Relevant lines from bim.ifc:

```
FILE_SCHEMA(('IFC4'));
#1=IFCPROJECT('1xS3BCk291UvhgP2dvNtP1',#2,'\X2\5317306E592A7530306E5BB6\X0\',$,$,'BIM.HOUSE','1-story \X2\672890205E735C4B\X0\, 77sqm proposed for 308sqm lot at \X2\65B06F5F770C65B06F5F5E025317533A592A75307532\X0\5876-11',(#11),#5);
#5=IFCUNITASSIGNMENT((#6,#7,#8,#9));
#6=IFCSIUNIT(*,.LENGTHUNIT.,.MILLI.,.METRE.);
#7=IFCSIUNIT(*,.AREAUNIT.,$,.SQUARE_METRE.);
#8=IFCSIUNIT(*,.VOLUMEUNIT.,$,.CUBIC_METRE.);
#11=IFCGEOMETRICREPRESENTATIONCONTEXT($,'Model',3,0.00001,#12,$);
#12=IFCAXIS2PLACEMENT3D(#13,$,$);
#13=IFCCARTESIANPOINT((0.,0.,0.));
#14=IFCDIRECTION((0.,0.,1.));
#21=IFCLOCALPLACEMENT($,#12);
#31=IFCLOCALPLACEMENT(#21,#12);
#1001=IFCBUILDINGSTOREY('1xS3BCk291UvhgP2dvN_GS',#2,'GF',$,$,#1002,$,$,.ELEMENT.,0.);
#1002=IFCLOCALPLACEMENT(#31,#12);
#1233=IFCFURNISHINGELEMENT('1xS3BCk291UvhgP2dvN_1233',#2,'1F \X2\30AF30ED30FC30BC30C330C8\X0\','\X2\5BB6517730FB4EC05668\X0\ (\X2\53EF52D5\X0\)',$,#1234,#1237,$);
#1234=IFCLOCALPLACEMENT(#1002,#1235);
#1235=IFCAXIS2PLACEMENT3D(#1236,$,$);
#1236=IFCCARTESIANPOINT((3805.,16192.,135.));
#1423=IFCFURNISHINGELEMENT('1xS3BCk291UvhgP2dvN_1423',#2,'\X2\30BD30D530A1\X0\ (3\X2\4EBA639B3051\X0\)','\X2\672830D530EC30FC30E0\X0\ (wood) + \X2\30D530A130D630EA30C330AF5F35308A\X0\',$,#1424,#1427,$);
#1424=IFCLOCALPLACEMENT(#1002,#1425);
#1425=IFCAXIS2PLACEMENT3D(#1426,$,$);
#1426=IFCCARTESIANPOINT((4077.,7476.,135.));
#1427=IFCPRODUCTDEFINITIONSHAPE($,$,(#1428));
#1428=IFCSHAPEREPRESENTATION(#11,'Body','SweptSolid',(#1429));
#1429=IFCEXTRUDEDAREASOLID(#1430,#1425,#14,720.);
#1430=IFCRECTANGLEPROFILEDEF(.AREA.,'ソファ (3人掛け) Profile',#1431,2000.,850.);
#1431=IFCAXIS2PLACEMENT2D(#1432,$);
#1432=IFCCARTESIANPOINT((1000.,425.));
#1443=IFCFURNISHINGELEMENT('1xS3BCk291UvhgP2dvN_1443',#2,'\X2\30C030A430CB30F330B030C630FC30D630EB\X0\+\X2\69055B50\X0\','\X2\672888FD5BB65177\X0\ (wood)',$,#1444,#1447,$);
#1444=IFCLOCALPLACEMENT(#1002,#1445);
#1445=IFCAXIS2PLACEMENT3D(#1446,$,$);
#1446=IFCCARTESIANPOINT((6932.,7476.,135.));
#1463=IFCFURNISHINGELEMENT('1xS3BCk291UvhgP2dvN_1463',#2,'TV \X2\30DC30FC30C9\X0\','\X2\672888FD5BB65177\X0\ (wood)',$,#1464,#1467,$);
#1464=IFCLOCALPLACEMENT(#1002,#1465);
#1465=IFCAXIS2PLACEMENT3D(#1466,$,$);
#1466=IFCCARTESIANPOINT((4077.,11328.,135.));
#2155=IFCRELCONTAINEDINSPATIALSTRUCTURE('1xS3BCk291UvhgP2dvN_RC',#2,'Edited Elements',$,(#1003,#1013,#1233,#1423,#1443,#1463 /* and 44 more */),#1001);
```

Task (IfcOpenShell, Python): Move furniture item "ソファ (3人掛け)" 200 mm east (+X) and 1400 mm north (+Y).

```python
import ifcopenshell
import ifcopenshell.api.geometry
import ifcopenshell.util.placement
import ifcopenshell.util.unit

model = ifcopenshell.open("bim.ifc")
unit_scale = ifcopenshell.util.unit.calculate_unit_scale(model)

item = model.by_guid("1xS3BCk291UvhgP2dvN_1423")
matrix = ifcopenshell.util.placement.get_local_placement(item.ObjectPlacement)
matrix[0, 3] += 0.2 / unit_scale
matrix[1, 3] += 1.4 / unit_scale
ifcopenshell.api.geometry.edit_object_placement(model, product=item, matrix=matrix, is_si=False)

print(ifcopenshell.util.placement.get_local_placement(item.ObjectPlacement).round(3) + 0.0)

model.write("bim_edited.ifc")
```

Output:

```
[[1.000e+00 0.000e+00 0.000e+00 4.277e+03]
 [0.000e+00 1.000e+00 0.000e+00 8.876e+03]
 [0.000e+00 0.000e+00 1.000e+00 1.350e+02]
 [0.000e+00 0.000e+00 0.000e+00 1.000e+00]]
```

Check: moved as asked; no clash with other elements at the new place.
